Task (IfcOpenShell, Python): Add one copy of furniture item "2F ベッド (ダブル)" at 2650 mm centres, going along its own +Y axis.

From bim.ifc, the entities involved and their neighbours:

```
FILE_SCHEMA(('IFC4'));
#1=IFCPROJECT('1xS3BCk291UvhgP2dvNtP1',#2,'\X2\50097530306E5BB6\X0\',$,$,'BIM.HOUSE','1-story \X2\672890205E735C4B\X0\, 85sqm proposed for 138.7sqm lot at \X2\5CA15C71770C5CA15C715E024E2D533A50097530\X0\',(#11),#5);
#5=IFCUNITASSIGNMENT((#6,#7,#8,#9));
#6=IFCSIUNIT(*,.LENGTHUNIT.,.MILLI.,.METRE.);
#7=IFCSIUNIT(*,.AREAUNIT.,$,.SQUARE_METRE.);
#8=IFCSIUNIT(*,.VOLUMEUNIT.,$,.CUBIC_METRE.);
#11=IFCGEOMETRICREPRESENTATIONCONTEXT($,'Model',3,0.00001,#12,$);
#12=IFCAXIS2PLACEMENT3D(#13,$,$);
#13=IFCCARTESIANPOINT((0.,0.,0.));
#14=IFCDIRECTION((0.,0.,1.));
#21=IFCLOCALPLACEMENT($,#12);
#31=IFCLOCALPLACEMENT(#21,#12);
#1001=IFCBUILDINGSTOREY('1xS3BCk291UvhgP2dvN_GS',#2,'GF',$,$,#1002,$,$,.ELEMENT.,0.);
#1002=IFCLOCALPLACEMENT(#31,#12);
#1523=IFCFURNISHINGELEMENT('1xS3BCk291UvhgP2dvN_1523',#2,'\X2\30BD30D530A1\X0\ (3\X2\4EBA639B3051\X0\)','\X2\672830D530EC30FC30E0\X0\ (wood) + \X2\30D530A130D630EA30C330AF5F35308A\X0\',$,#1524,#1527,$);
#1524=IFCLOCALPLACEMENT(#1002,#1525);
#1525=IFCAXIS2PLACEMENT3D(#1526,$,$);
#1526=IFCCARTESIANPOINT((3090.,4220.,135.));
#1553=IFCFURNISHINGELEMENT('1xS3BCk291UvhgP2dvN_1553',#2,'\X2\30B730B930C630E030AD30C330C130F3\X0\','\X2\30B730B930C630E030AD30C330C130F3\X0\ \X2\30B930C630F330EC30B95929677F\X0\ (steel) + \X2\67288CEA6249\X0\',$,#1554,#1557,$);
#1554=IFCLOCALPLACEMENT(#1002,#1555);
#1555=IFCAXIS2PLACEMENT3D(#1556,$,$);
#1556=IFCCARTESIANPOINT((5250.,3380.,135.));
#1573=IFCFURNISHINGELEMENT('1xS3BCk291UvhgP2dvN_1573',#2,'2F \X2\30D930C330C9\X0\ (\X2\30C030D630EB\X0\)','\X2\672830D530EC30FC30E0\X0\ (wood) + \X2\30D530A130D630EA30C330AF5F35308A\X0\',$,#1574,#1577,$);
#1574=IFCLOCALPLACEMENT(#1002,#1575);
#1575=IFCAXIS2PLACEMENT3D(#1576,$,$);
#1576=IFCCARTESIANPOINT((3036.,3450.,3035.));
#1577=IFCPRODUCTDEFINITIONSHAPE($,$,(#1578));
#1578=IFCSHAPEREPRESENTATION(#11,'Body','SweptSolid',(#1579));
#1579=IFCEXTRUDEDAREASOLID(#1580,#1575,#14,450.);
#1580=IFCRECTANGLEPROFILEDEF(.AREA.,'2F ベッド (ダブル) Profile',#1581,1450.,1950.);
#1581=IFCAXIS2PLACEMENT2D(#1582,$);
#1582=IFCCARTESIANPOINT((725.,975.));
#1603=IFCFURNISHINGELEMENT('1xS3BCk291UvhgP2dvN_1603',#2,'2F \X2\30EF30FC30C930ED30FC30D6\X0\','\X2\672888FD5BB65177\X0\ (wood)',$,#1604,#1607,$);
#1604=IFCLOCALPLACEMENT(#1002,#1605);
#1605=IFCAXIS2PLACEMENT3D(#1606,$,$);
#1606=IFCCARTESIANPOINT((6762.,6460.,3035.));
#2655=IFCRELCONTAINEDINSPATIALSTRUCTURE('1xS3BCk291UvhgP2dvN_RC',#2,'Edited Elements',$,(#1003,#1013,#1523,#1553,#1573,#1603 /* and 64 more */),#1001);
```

```python
import ifcopenshell
import ifcopenshell.api.geometry
import ifcopenshell.api.root
import ifcopenshell.util.element
import ifcopenshell.util.placement

model = ifcopenshell.open("bim.ifc")


def reuse_history(source, copy):
    """copy_class also copies each property set's owner history, people and application; keep the originals."""
    for rel in copy.IsDefinedBy:
        if rel.is_a("IfcRelDefinesByProperties") and (history := rel.RelatingPropertyDefinition.OwnerHistory):
            rel.RelatingPropertyDefinition.OwnerHistory = source.OwnerHistory
            ifcopenshell.util.element.remove_deep2(model, history)


source = model.by_guid("1xS3BCk291UvhgP2dvN_1573")
base = ifcopenshell.util.placement.get_local_placement(source.ObjectPlacement)
step = base[:3, 1] * 2650.0

for i in range(1, 2):
    copy = ifcopenshell.api.root.copy_class(model, product=source)
    copy.Representation = ifcopenshell.util.element.copy_deep(
        model, source.Representation, exclude=["IfcGeometricRepresentationContext", "IfcRepresentationMap"]
    )
    reuse_history(source, copy)
    matrix = base.copy()
    matrix[:3, 3] += i * step
    print("added at", matrix[:3, 3].round(3) + 0.0)
    ifcopenshell.api.geometry.edit_object_placement(model, product=copy, matrix=matrix, is_si=False)

model.write("bim-out.ifc")
```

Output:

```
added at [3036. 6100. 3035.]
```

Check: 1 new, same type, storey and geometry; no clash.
